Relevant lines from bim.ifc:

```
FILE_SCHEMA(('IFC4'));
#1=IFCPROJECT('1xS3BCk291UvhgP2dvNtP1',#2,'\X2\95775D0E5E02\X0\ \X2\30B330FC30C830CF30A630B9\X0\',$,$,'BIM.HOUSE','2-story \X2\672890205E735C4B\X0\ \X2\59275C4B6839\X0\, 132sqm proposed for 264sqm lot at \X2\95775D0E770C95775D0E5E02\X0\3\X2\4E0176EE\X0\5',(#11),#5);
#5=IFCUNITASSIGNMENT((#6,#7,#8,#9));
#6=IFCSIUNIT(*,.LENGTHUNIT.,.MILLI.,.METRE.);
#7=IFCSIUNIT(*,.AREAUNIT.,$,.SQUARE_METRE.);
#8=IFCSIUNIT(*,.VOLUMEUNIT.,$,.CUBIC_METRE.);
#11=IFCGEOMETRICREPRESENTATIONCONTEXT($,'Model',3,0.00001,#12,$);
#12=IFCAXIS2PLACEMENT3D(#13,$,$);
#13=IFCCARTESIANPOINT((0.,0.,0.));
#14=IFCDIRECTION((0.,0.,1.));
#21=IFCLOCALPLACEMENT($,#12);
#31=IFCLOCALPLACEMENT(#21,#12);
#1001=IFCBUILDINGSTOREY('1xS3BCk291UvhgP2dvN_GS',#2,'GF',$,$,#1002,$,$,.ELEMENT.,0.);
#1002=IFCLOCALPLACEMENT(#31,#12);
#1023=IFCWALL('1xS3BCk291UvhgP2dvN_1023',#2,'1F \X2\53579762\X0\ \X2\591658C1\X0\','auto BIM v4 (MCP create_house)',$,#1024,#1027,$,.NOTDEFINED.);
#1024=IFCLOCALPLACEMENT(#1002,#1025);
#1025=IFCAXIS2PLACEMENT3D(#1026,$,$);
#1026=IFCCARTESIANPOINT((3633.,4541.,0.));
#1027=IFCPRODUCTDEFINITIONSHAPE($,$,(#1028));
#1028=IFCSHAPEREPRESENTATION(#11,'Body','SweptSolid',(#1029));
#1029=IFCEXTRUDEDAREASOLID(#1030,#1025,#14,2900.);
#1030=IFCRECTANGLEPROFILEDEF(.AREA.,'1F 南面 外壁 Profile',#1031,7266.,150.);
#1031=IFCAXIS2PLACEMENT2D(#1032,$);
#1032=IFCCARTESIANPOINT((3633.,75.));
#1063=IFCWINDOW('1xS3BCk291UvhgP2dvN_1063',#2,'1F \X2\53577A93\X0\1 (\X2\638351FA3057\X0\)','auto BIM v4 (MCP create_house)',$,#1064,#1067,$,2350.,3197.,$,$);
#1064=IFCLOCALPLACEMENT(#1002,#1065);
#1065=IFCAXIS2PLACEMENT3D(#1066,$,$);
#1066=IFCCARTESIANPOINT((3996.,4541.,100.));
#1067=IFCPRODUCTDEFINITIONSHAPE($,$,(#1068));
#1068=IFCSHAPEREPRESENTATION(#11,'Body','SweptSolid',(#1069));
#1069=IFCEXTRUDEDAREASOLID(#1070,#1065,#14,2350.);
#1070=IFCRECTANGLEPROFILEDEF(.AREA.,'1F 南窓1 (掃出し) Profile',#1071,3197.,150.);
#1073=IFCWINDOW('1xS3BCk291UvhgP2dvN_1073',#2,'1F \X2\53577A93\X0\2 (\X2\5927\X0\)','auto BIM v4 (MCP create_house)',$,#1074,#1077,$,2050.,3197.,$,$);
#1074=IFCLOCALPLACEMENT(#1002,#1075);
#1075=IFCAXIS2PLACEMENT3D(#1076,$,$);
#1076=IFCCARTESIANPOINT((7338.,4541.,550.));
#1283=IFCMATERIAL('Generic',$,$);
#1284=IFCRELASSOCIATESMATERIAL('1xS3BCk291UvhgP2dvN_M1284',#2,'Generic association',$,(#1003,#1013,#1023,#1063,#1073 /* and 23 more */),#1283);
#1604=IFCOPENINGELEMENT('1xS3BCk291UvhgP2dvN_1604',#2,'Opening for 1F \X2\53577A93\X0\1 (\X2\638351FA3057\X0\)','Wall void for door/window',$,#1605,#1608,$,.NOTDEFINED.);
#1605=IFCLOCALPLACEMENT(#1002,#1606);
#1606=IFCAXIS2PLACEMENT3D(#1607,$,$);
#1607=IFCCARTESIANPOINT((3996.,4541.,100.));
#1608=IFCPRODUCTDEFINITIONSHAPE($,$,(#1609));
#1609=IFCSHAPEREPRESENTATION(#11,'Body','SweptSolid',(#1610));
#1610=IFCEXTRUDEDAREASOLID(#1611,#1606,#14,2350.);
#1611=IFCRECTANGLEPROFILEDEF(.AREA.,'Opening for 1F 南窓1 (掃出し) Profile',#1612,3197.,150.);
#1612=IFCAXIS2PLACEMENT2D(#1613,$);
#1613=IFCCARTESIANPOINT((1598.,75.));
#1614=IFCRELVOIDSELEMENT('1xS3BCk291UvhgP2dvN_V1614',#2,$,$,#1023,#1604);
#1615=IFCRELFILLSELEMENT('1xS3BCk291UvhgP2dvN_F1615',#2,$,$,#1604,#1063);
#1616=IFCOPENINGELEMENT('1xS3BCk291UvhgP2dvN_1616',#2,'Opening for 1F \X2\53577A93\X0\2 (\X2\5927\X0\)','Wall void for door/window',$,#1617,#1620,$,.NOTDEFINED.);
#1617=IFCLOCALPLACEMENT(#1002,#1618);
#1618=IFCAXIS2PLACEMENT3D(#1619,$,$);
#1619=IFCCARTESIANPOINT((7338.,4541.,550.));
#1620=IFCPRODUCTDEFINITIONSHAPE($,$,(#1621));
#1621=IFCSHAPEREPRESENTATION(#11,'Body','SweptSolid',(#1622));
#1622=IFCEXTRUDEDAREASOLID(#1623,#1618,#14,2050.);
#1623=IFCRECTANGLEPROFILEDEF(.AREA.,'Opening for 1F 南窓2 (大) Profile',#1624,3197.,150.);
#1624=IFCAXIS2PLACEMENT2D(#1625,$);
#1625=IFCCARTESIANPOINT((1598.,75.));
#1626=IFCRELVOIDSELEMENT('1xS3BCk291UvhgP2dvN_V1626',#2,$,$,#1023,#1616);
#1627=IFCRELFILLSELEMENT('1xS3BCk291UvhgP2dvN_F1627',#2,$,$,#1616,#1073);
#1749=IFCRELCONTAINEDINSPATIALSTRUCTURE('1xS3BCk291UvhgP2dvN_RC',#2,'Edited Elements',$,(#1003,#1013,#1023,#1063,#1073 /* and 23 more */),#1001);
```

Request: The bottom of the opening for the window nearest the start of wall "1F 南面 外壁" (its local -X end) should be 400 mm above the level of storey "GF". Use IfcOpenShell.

```python
import numpy as np
import ifcopenshell
import ifcopenshell.api.geometry
import ifcopenshell.geom
import ifcopenshell.util.element
import ifcopenshell.util.placement
import ifcopenshell.util.shape
import ifcopenshell.util.unit

model = ifcopenshell.open("bim.ifc")
unit_scale = ifcopenshell.util.unit.calculate_unit_scale(model)

window = model.by_guid("1xS3BCk291UvhgP2dvN_1063")
opening = window.FillsVoids[0].RelatingOpeningElement
storey = ifcopenshell.util.element.get_container(window, ifc_class="IfcBuildingStorey")
level = ifcopenshell.util.placement.get_local_placement(storey.ObjectPlacement)[2, 3]

# The opening's origin need not be at the sill, so measure its lowest point.
shape = ifcopenshell.geom.create_shape(ifcopenshell.geom.settings(), opening)
bottom = ifcopenshell.util.shape.get_shape_bottom_elevation(shape, shape.geometry) / unit_scale
dz = level + 0.4 / unit_scale - bottom

shift = np.array([0.0, 0.0, dz])
# The window is not placed relative to its opening, so move both.
for product in (opening, window):
    matrix = ifcopenshell.util.placement.get_local_placement(product.ObjectPlacement)
    matrix[:3, 3] += shift
    ifcopenshell.api.geometry.edit_object_placement(model, product=product, matrix=matrix, is_si=False)

print(f"moved by {dz * unit_scale:+.3f} m")

model.write("bim_v2.ifc")
```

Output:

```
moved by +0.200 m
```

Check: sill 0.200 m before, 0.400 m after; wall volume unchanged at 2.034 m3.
